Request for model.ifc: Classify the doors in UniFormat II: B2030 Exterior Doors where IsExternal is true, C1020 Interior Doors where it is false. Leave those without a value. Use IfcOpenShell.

First a look at what the model holds.

```python
import ifcopenshell
import ifcopenshell.util.element

model = ifcopenshell.open("model.ifc")
print(model.schema)
print("classifications:", [c.Name for c in model.by_type("IfcClassification")])
values = [ifcopenshell.util.element.get_pset(e, "Pset_DoorCommon", "IsExternal") for e in model.by_type("IfcDoor")]
for value in (True, False, None):
    print("IsExternal", value, values.count(value))
```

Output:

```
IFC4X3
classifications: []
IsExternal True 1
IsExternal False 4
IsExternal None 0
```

```python
import ifcopenshell
import ifcopenshell.api.classification
import ifcopenshell.util.element

model = ifcopenshell.open("model.ifc")

system = ifcopenshell.api.classification.add_classification(model, classification="UniFormat II")

doors = model.by_type("IfcDoor")
external = {e: ifcopenshell.util.element.get_pset(e, "Pset_DoorCommon", "IsExternal") for e in doors}
for flag, code, name in ((True, "B2030", "Exterior Doors"), (False, "C1020", "Interior Doors")):
    products = [e for e in doors if external[e] is flag]
    ifcopenshell.api.classification.add_reference(
        model, products=products, classification=system, identification=code, name=name
    )
    print(code, len(products))

model.write("model_rev.ifc")
```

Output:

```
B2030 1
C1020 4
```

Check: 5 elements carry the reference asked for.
